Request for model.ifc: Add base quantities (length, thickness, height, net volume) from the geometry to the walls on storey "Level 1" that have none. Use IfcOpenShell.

First a look at what the model holds.

```python
import ifcopenshell
import ifcopenshell.util.element
import ifcopenshell.util.unit

model = ifcopenshell.open("model.ifc")
print(model.schema)
for unit_type in ("LENGTHUNIT", "AREAUNIT", "VOLUMEUNIT"):
    print(unit_type, ifcopenshell.util.unit.calculate_unit_scale(model, unit_type))
storey = next(s for s in model.by_type("IfcBuildingStorey") if s.Name == "Level 1")
walls = [e for e in ifcopenshell.util.element.get_decomposition(storey) if e.is_a("IfcWall")]
for e in sorted(walls, key=lambda e: e.id()):
    print(e.id(), e.is_a(), e.Name, list(ifcopenshell.util.element.get_psets(e, qtos_only=True)), sep=" | ")
```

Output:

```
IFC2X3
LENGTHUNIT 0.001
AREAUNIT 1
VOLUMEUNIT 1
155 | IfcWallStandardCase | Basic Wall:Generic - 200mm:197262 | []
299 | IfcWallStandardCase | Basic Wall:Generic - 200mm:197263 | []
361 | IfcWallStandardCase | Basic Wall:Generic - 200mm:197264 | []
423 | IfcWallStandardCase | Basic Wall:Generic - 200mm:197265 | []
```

```python
import ifcopenshell
import ifcopenshell.api.pset
import ifcopenshell.geom
import ifcopenshell.util.element
import ifcopenshell.util.shape
import ifcopenshell.util.unit

model = ifcopenshell.open("model.ifc")
unit_scale = ifcopenshell.util.unit.calculate_unit_scale(model)
volume_scale = ifcopenshell.util.unit.calculate_unit_scale(model, "VOLUMEUNIT")
settings = ifcopenshell.geom.settings()

storey = next(s for s in model.by_type("IfcBuildingStorey") if s.Name == "Level 1")
walls = [e for e in ifcopenshell.util.element.get_decomposition(storey) if e.is_a("IfcWall")]

for e in sorted(walls, key=lambda e: e.id()):
    if ifcopenshell.util.element.get_psets(e, qtos_only=True, should_inherit=False):
        continue
    # Geometry comes back in metres, in the element's own axes.
    shape = ifcopenshell.geom.create_shape(settings, e)
    values = {
        "Length": ifcopenshell.util.shape.get_x(shape.geometry) / unit_scale,
        "Width": ifcopenshell.util.shape.get_y(shape.geometry) / unit_scale,
        "Height": ifcopenshell.util.shape.get_z(shape.geometry) / unit_scale,
        "NetVolume": ifcopenshell.util.shape.get_volume(shape.geometry) / volume_scale,
    }
    qto = ifcopenshell.api.pset.add_qto(model, product=e, name="BaseQuantities")
    ifcopenshell.api.pset.edit_qto(model, qto=qto, properties=values)
    print(e.id(), {k: round(v, 3) for k, v in values.items()})

model.write("model_updated.ifc")
```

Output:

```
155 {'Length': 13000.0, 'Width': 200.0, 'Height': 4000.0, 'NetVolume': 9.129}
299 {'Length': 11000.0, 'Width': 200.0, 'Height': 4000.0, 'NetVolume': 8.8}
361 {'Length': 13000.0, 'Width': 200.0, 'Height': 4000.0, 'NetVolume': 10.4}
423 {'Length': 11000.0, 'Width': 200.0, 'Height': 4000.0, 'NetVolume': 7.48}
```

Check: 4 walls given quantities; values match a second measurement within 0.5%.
